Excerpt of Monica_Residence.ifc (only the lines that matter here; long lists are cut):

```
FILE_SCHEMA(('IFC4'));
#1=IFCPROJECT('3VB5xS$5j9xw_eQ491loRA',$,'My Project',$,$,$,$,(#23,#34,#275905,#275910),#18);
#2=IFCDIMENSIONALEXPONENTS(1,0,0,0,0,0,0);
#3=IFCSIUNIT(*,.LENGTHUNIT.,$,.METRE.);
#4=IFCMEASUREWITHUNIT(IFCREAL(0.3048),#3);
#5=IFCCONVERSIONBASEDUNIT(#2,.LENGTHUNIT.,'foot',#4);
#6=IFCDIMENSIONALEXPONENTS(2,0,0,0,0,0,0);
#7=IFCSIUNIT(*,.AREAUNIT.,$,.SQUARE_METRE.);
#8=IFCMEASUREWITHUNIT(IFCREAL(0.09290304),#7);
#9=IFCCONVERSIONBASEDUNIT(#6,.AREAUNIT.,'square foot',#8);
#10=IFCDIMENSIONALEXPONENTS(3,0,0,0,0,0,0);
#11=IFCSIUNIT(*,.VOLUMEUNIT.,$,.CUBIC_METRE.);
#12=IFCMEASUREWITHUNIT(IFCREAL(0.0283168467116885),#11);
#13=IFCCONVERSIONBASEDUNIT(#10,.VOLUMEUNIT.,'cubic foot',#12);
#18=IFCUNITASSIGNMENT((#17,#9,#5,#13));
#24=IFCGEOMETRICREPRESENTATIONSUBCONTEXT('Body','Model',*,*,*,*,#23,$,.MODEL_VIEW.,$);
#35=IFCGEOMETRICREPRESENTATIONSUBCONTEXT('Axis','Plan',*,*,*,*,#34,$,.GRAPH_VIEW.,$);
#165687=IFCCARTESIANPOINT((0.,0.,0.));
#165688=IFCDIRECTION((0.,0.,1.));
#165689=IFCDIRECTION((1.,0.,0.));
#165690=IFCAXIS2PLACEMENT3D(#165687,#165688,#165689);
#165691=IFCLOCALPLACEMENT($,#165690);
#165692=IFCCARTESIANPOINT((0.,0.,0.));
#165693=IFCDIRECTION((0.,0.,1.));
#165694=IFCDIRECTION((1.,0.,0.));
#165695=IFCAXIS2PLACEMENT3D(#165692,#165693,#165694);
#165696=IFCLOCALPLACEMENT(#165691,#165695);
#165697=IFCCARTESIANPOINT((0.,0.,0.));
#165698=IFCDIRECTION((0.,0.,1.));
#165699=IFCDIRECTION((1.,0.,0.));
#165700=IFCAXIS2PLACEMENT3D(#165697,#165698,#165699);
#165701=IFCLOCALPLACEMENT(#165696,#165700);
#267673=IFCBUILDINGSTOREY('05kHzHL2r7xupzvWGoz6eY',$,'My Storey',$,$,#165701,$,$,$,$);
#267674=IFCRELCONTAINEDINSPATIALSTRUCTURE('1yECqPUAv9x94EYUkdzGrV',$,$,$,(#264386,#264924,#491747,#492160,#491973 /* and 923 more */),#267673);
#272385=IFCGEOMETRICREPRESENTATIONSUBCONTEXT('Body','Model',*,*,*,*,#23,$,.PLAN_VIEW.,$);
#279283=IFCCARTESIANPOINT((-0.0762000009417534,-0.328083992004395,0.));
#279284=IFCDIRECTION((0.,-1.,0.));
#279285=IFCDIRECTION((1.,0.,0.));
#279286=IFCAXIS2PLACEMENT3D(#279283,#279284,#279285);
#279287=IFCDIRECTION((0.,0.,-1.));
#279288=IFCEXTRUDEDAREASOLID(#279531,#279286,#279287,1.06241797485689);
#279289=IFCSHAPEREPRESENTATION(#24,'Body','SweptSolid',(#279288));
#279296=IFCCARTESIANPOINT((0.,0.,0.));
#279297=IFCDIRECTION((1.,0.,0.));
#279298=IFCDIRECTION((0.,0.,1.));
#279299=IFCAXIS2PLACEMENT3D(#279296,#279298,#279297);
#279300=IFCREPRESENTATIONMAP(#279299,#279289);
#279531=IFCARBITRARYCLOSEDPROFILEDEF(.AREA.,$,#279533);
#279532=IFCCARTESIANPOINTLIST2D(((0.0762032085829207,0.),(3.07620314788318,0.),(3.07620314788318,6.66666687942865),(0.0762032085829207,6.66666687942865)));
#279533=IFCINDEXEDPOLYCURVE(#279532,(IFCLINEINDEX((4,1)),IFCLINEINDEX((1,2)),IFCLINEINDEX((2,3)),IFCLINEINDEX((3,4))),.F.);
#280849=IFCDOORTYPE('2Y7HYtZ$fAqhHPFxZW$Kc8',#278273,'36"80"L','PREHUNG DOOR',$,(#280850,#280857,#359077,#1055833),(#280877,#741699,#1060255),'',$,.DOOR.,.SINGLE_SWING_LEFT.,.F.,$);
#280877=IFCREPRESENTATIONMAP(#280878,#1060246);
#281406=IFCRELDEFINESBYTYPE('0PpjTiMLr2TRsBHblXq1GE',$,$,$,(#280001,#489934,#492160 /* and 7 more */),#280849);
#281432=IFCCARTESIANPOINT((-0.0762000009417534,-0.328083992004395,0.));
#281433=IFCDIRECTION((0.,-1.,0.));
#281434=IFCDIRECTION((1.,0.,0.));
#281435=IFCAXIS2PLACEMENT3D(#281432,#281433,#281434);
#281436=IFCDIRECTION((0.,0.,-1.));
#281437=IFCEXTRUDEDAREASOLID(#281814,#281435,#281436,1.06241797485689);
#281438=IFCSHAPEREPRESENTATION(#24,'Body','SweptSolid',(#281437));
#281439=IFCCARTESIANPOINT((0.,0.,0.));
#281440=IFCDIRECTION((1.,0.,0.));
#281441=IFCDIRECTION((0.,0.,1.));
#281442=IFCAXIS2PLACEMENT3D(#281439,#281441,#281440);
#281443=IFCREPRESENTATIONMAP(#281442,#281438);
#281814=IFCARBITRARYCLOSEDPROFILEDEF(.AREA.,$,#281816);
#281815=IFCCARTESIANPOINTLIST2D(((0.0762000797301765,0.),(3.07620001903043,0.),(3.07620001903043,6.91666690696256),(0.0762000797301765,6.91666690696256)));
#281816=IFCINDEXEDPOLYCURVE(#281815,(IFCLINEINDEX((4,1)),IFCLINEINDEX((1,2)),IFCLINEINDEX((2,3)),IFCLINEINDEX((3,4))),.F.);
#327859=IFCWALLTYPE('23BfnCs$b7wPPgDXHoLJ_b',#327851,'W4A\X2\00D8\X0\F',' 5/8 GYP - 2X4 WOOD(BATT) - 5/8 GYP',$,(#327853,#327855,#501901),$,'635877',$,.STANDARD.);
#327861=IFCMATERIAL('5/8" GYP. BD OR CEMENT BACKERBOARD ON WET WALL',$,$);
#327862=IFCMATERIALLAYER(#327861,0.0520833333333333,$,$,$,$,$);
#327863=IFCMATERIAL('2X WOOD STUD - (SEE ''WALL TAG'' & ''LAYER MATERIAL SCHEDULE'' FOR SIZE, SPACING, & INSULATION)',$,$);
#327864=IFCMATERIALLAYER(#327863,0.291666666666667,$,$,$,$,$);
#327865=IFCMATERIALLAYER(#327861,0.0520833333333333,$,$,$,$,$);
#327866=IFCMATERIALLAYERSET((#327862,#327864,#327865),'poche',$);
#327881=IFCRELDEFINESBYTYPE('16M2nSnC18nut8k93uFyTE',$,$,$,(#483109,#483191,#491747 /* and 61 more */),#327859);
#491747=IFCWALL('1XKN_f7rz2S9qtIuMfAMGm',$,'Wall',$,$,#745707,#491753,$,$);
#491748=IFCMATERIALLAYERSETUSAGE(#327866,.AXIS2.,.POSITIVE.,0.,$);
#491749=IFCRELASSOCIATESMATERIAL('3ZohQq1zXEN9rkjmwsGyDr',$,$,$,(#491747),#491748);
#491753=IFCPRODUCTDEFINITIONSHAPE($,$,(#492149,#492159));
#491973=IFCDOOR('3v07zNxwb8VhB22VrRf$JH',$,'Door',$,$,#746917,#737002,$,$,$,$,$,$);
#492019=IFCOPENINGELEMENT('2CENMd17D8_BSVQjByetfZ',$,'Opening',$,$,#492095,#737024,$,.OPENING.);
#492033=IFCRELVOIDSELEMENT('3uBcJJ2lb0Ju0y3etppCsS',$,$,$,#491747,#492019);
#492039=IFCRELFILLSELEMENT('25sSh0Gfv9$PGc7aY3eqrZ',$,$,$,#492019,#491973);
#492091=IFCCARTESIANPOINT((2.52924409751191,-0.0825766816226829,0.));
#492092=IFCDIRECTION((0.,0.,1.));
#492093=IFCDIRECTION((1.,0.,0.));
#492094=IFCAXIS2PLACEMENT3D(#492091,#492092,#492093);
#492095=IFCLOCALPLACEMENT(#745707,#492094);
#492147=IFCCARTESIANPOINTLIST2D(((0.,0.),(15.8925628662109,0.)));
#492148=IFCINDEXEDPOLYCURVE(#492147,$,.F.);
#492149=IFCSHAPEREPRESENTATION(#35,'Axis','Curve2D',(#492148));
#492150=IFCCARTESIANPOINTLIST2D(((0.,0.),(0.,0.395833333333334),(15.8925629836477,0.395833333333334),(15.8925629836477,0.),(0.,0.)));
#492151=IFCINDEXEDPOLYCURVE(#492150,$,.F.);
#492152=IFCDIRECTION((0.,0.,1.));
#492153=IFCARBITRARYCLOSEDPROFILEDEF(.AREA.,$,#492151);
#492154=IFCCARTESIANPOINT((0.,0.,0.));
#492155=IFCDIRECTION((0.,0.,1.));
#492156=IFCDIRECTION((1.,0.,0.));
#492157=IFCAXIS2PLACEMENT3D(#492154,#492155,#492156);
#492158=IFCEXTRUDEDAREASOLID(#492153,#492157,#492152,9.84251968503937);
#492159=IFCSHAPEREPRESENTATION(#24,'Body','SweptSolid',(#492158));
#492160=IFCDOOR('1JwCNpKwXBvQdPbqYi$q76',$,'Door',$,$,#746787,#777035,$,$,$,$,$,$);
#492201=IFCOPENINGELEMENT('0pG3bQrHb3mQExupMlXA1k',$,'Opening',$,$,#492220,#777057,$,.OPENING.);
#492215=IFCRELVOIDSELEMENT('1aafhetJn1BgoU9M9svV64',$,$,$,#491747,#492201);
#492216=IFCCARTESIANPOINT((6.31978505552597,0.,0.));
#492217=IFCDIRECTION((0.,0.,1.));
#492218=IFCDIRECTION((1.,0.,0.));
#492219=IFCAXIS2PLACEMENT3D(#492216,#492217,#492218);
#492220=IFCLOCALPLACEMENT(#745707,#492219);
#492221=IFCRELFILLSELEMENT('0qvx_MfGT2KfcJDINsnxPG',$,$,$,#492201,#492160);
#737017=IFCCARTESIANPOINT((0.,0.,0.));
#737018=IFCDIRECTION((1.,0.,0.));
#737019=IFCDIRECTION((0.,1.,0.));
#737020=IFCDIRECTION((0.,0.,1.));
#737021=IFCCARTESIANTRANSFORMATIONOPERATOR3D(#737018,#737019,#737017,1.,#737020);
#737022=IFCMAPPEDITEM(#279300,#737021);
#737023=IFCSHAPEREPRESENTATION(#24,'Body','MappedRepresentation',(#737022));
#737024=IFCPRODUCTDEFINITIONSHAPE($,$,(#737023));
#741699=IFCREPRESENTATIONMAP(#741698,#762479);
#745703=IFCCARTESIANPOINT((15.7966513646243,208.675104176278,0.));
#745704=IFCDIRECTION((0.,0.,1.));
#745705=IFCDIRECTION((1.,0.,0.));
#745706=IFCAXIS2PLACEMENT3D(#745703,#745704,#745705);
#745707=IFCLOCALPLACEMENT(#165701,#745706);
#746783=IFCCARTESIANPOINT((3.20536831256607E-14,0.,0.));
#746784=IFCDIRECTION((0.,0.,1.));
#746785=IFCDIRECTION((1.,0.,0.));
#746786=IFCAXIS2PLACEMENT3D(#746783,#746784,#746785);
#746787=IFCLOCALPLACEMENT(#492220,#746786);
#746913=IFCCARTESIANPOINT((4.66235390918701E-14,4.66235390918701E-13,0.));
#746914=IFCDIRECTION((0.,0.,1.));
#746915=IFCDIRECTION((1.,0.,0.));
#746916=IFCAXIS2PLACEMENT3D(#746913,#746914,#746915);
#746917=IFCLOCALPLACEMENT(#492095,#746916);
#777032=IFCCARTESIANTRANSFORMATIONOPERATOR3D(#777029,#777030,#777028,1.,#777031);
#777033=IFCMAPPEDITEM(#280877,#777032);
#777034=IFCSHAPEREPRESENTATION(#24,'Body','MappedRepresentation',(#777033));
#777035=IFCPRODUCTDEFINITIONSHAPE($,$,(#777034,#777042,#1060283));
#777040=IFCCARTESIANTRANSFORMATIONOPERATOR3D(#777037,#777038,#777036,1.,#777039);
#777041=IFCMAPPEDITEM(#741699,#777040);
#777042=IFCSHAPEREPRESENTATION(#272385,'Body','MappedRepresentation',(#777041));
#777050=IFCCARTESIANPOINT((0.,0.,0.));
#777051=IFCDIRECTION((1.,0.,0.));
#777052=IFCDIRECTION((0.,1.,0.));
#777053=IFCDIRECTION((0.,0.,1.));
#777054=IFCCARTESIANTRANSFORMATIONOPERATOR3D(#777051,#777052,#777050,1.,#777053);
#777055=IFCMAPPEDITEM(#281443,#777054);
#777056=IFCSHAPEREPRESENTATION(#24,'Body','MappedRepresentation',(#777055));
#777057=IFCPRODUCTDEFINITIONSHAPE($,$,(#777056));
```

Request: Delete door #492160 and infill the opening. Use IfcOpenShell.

```python
import ifcopenshell
import ifcopenshell.api.feature
import ifcopenshell.api.root
import ifcopenshell.geom
import ifcopenshell.util.shape

model = ifcopenshell.open("Monica_Residence.ifc")
settings = ifcopenshell.geom.settings()


def volume(element):
    """Net volume in cubic metres, openings subtracted."""
    shape = ifcopenshell.geom.create_shape(settings, element)
    return ifcopenshell.util.shape.get_volume(shape.geometry)


door = model.by_id(492160)
opening = door.FillsVoids[0].RelatingOpeningElement
wall = opening.VoidsElements[0].RelatingBuildingElement
before = volume(wall)

ifcopenshell.api.root.remove_product(model, product=door)
ifcopenshell.api.feature.remove_feature(model, feature=opening)

after = volume(wall)

print(f"wall volume {before:.3f} -> {after:.3f} m3")

model.write("Monica_Residence_edited.ifc")
```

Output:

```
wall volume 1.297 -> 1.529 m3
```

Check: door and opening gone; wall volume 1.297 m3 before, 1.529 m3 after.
